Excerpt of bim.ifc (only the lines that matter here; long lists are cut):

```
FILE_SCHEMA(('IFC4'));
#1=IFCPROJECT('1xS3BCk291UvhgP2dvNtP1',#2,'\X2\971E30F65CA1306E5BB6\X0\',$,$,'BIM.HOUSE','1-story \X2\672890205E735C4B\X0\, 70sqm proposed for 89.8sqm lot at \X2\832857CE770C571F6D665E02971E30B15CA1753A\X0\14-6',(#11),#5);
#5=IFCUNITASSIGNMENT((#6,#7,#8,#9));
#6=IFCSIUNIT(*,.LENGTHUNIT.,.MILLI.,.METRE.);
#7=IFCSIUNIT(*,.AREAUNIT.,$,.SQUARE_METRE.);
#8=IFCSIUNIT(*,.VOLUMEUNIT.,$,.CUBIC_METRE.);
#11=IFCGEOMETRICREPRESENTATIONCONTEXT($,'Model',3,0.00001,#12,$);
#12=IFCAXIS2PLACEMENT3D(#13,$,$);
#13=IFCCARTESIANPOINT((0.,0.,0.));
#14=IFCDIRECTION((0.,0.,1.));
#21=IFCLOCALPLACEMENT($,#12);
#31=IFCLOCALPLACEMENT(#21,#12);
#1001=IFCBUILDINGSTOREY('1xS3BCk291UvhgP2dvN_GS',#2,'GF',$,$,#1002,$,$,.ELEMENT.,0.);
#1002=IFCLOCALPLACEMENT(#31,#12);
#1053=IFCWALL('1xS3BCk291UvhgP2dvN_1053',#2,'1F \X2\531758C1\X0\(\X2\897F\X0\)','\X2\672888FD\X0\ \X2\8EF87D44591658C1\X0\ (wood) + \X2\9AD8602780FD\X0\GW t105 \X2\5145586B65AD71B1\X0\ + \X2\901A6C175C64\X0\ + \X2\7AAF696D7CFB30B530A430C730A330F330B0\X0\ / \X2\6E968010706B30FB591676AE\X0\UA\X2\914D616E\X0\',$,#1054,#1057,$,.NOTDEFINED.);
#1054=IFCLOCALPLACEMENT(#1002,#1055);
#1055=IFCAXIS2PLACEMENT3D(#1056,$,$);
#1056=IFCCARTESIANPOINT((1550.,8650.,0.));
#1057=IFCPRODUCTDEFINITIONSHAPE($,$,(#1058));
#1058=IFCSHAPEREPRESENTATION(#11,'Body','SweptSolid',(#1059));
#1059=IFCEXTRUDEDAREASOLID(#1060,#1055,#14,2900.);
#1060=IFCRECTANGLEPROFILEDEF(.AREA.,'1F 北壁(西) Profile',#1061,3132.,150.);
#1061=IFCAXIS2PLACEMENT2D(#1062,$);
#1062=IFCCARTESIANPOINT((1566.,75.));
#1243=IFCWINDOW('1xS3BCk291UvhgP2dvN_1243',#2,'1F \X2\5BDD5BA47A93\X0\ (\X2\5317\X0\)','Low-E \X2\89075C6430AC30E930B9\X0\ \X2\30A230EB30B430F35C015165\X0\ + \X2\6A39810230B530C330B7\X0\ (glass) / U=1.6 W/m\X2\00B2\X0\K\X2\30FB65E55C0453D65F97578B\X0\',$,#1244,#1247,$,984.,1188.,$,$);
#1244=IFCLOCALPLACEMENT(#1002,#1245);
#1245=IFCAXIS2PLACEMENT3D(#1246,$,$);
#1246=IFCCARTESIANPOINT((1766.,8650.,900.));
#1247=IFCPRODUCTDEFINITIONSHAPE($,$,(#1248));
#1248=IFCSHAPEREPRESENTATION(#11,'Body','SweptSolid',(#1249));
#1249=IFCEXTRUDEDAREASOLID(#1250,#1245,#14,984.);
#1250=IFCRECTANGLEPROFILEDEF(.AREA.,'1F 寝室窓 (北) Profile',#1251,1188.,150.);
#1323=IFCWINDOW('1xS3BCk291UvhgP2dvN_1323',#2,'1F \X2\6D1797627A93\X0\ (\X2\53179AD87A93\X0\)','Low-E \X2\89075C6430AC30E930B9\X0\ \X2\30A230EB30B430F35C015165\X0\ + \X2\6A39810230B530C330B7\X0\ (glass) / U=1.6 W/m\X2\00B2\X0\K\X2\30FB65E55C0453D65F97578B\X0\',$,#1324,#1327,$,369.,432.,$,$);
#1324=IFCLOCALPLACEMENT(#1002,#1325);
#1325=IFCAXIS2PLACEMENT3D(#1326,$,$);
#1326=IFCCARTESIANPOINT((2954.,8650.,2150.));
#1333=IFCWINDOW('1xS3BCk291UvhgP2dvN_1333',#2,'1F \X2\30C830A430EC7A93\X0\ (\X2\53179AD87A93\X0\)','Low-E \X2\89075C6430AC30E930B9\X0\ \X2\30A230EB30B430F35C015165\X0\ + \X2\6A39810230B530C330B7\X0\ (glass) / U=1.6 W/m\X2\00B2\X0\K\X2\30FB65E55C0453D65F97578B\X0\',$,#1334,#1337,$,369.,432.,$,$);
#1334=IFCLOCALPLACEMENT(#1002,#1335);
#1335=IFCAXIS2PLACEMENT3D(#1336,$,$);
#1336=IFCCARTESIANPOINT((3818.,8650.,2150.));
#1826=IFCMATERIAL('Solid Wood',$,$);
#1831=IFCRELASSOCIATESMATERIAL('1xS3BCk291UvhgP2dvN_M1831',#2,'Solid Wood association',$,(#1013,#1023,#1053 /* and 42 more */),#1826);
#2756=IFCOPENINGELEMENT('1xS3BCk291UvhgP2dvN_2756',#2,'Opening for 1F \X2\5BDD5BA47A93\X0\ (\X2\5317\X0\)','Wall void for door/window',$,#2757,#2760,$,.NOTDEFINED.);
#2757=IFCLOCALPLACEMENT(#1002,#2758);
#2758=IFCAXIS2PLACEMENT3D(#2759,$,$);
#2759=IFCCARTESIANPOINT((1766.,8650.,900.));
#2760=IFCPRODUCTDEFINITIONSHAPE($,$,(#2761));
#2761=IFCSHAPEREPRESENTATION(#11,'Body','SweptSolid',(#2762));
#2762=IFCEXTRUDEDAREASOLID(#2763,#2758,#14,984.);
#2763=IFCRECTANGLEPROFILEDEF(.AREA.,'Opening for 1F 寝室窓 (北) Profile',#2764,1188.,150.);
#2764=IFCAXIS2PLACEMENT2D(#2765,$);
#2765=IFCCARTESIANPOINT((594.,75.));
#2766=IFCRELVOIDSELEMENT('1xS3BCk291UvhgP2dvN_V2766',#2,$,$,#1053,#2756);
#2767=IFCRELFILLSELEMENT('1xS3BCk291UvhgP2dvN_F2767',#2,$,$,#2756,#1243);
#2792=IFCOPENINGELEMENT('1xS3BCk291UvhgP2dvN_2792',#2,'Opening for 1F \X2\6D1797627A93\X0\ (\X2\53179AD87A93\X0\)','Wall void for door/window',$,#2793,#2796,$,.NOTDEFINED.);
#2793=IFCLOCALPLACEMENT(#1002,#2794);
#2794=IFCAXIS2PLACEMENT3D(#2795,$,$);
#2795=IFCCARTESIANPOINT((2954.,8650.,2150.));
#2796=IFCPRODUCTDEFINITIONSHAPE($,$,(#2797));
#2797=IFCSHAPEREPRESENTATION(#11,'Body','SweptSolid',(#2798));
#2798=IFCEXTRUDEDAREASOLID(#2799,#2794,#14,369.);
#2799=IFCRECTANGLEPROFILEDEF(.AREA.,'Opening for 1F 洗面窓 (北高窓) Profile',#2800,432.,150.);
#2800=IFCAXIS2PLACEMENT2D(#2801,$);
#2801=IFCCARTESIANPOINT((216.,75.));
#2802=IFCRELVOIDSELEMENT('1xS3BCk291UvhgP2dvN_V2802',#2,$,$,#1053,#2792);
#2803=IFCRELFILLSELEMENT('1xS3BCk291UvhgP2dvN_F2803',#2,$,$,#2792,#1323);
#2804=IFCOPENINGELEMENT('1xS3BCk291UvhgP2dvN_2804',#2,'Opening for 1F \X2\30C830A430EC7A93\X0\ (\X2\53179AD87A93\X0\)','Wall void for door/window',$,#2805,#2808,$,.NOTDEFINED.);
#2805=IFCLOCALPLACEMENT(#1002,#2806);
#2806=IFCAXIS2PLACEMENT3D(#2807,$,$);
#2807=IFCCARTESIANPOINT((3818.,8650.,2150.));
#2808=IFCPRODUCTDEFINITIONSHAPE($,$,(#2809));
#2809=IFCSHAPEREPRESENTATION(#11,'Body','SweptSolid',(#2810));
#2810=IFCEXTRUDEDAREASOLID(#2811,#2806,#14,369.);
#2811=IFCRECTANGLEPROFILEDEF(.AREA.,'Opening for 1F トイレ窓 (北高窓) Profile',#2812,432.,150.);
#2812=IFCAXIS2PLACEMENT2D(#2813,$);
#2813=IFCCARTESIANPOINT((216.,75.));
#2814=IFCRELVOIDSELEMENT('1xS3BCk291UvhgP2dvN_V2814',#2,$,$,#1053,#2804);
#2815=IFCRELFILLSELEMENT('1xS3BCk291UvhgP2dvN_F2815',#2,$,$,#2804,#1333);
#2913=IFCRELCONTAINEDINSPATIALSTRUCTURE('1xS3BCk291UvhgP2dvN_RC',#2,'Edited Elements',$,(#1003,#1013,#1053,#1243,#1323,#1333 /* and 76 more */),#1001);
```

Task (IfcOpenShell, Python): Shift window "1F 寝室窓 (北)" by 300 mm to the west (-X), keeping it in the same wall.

```python
import ifcopenshell
import ifcopenshell.api.geometry
import ifcopenshell.util.placement
import ifcopenshell.util.unit

model = ifcopenshell.open("bim.ifc")
unit_scale = ifcopenshell.util.unit.calculate_unit_scale(model)

window = model.by_guid("1xS3BCk291UvhgP2dvN_1243")
opening = window.FillsVoids[0].RelatingOpeningElement
wall = opening.VoidsElements[0].RelatingBuildingElement

wall_matrix = ifcopenshell.util.placement.get_local_placement(wall.ObjectPlacement)
shift = wall_matrix[:3, 0] * -0.3 / unit_scale
before = ifcopenshell.util.placement.get_local_placement(window.ObjectPlacement)[:3, 3].copy()

# The window is not placed relative to its opening, so move both.
for product in (opening, window):
    matrix = ifcopenshell.util.placement.get_local_placement(product.ObjectPlacement)
    matrix[:3, 3] += shift
    ifcopenshell.api.geometry.edit_object_placement(model, product=product, matrix=matrix, is_si=False)

after = ifcopenshell.util.placement.get_local_placement(window.ObjectPlacement)[:3, 3]
print("window moved by", (after - before).round(3) + 0.0)

model.write("bim_rev.ifc")
```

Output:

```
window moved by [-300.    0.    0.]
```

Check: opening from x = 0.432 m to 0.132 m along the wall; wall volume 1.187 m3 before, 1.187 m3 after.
